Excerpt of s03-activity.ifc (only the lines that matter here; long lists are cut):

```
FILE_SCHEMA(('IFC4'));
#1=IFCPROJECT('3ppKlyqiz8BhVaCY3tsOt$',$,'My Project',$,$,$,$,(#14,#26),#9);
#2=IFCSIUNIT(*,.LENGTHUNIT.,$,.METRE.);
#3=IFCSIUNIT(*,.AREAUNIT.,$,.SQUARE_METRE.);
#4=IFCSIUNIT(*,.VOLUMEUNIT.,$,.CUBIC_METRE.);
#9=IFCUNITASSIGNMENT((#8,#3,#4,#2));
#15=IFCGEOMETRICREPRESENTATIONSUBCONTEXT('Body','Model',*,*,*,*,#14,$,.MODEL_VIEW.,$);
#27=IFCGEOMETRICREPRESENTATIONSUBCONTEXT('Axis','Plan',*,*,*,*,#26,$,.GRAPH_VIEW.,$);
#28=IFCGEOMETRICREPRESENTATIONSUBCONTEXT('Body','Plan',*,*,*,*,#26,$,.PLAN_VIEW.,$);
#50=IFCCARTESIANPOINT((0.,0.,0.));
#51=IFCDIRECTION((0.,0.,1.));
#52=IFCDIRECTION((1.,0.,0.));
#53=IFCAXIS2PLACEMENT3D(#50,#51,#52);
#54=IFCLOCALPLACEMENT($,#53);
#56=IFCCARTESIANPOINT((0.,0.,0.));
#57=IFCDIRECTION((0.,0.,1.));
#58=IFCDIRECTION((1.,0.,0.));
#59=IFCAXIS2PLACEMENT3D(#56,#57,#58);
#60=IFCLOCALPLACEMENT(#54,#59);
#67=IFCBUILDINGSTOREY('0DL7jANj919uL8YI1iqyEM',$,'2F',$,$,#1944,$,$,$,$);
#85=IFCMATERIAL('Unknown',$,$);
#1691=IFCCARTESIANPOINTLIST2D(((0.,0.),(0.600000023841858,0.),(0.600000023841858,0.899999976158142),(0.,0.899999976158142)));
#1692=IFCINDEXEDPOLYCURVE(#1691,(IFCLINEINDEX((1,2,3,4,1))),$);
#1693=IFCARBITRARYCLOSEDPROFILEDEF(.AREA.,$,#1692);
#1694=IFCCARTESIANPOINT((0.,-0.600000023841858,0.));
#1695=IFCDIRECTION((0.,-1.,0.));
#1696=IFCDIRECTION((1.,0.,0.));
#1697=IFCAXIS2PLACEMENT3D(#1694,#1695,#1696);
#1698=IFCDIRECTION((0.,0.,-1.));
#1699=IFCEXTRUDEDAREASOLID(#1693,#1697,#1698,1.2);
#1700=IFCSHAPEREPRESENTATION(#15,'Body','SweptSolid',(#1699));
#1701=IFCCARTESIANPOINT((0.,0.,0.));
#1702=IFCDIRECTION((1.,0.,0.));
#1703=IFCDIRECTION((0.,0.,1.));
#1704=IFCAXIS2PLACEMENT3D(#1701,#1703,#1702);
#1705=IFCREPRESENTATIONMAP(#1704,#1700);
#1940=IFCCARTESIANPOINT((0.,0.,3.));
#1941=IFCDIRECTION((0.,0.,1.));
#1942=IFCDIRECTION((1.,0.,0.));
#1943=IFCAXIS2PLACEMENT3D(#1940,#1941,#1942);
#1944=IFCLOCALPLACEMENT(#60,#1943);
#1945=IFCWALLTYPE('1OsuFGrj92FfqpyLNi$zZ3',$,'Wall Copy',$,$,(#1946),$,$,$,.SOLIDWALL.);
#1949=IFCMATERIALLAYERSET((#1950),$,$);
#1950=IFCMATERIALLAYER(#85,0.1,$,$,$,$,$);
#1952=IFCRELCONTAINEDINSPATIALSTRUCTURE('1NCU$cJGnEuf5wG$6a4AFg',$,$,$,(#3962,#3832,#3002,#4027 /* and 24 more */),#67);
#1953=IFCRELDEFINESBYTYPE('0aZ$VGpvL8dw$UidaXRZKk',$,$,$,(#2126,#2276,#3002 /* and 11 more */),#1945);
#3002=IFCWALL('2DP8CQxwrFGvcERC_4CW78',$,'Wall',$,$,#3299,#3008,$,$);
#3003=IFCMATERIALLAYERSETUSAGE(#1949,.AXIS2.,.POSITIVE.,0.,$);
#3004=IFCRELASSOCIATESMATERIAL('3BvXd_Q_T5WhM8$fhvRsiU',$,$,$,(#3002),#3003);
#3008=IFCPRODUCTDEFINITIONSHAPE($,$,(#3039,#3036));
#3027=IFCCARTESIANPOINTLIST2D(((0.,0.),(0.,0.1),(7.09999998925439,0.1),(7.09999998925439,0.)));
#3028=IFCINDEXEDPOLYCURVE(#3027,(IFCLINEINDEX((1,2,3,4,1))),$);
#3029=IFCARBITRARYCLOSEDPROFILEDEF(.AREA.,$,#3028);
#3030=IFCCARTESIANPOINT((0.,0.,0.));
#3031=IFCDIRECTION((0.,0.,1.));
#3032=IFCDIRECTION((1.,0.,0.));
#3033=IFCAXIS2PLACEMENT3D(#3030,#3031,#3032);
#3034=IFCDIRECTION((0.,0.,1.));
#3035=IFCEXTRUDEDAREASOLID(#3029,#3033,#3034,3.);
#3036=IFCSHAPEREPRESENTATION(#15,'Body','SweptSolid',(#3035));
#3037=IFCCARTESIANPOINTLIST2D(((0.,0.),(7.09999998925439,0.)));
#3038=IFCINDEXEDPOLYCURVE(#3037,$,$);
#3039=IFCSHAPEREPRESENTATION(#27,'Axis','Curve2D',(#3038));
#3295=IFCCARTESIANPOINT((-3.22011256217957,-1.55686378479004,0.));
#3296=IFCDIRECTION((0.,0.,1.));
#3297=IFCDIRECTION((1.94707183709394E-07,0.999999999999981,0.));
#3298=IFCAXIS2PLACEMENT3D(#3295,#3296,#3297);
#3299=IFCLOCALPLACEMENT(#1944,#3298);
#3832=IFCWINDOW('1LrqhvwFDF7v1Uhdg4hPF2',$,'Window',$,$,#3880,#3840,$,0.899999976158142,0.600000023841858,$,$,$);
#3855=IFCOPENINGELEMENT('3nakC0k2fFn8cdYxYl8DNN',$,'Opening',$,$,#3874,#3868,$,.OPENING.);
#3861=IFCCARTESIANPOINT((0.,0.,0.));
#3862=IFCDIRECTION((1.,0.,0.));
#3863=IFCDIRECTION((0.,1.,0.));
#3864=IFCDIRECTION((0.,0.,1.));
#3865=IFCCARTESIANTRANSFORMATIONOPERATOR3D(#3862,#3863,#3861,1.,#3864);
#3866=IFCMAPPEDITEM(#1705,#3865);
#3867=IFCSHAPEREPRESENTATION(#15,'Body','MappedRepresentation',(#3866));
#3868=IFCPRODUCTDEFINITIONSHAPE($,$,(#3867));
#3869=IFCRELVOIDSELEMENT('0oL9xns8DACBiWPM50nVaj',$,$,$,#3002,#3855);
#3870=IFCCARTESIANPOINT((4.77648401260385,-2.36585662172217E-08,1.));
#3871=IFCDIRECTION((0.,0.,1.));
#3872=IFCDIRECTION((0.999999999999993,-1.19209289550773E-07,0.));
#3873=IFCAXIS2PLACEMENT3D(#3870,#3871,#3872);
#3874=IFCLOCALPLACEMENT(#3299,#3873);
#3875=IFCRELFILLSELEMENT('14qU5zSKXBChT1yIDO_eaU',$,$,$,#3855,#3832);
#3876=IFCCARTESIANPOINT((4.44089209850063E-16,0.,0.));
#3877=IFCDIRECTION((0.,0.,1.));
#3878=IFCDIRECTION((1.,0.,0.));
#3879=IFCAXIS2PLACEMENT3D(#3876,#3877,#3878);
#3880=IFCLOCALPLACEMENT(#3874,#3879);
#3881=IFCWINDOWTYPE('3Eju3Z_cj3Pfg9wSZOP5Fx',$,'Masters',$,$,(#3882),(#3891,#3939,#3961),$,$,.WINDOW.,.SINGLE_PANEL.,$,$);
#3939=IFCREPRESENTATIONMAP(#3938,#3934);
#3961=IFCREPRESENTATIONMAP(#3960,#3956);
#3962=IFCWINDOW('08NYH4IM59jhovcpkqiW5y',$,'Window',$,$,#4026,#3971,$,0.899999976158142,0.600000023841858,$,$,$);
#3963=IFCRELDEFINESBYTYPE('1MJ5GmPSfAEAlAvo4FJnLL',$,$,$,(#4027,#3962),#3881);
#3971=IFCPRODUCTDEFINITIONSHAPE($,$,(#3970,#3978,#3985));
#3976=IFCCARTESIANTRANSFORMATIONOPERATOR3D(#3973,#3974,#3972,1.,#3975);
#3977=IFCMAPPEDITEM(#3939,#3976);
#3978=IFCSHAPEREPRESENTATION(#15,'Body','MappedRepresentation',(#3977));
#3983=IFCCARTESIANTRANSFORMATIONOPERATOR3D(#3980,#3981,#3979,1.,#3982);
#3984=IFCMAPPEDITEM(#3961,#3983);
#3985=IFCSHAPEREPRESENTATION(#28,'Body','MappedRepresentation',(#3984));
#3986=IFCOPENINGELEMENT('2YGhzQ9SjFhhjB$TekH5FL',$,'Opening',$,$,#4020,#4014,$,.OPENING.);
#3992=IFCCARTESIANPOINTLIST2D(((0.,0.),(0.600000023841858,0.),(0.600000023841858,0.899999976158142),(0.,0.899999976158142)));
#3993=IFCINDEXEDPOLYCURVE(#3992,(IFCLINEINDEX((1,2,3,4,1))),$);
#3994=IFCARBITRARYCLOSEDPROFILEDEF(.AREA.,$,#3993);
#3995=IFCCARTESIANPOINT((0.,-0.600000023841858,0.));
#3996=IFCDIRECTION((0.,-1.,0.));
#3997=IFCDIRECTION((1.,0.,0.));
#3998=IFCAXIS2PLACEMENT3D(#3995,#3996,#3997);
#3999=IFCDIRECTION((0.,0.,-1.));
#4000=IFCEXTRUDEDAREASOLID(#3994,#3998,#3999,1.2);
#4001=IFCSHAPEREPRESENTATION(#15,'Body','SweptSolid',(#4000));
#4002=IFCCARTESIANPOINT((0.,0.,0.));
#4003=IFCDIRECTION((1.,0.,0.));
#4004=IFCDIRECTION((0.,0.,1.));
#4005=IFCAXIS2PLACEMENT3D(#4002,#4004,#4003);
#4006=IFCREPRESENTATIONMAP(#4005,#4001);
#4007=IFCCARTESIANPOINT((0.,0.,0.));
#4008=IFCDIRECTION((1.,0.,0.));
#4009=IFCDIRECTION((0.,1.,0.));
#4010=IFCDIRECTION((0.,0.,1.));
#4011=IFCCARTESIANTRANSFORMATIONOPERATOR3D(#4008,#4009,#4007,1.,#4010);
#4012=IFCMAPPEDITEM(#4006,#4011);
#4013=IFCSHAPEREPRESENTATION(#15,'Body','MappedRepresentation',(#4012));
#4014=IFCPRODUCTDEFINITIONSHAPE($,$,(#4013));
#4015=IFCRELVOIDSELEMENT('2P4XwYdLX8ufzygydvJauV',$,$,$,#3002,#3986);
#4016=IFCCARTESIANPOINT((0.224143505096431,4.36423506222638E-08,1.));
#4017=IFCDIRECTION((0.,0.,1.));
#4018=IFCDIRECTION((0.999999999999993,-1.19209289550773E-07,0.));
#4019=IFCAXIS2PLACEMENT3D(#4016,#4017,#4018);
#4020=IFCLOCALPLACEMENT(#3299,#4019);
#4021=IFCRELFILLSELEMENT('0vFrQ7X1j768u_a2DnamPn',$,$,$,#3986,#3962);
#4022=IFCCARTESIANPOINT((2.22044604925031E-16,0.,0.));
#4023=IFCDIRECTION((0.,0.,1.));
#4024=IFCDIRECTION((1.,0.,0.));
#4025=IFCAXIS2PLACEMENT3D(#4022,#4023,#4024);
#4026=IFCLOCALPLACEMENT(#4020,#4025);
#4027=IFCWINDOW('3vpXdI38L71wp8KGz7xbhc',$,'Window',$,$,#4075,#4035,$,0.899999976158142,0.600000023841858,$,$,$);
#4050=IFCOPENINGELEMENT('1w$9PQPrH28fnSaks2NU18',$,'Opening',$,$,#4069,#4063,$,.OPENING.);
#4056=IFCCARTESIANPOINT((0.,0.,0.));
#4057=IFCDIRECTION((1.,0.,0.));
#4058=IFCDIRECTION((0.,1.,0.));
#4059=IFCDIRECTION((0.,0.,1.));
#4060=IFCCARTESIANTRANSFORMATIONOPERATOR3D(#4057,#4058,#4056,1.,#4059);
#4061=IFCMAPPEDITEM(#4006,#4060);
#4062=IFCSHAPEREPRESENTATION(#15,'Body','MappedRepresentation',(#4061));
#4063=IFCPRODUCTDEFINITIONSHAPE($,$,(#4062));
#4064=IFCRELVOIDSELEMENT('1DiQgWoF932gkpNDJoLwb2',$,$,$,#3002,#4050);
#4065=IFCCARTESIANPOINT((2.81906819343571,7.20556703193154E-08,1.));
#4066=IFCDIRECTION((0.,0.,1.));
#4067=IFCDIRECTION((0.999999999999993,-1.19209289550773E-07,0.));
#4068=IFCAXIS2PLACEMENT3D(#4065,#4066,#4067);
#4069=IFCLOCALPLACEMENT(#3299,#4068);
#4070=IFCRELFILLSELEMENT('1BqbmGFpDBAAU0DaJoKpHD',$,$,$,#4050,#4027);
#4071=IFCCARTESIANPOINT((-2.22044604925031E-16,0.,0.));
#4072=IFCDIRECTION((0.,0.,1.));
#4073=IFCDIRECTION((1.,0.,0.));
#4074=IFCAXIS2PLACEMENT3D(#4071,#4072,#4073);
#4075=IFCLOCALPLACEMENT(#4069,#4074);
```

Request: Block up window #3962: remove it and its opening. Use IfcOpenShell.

```python
import ifcopenshell
import ifcopenshell.api.feature
import ifcopenshell.api.root
import ifcopenshell.geom
import ifcopenshell.util.shape

model = ifcopenshell.open("s03-activity.ifc")
settings = ifcopenshell.geom.settings()


def volume(element):
    """Net volume in cubic metres, openings subtracted."""
    shape = ifcopenshell.geom.create_shape(settings, element)
    return ifcopenshell.util.shape.get_volume(shape.geometry)


window = model.by_id(3962)
opening = window.FillsVoids[0].RelatingOpeningElement
wall = opening.VoidsElements[0].RelatingBuildingElement
before = volume(wall)

ifcopenshell.api.root.remove_product(model, product=window)
ifcopenshell.api.feature.remove_feature(model, feature=opening)

after = volume(wall)

print(f"wall volume {before:.3f} -> {after:.3f} m3")

model.write("s03-activity-out.ifc")
```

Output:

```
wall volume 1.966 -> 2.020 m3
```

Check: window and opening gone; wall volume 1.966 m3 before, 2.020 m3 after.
